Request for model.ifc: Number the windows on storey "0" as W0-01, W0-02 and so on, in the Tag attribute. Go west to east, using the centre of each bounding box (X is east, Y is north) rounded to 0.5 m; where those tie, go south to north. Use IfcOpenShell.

First a look at what the model holds.

```python
import ifcopenshell
import ifcopenshell.util.element
import ifcopenshell.util.placement

model = ifcopenshell.open("model.ifc")
print(model.schema)
storey = next(s for s in model.by_type("IfcBuildingStorey") if s.Name == "0")
windows = [e for e in ifcopenshell.util.element.get_decomposition(storey) if e.is_a("IfcWindow")]
for e in sorted(windows, key=lambda e: e.id()):
    origin = ifcopenshell.util.placement.get_local_placement(e.ObjectPlacement)[:3, 3]
    print(e.id(), e.Tag, e.Name, origin.round(2) + 0.0, sep=" | ")
```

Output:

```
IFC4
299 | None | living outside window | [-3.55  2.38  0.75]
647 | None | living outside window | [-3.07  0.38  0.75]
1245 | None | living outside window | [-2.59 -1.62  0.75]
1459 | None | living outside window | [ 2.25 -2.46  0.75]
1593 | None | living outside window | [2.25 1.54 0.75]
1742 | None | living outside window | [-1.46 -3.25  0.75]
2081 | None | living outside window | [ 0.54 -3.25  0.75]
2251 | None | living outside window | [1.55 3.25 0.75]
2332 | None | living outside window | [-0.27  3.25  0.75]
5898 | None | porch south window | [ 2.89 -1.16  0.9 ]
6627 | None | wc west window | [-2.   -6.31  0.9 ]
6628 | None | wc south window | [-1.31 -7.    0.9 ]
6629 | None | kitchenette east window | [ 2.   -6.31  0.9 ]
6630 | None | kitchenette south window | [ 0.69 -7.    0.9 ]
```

```python
import ifcopenshell
import ifcopenshell.geom
import ifcopenshell.util.element
import ifcopenshell.util.shape

model = ifcopenshell.open("model.ifc")
settings = ifcopenshell.geom.settings()
settings.set("use-world-coords", True)


def centre(element):
    shape = ifcopenshell.geom.create_shape(settings, element)
    return ifcopenshell.util.shape.get_bbox_centroid(shape.geometry)


storey = next(s for s in model.by_type("IfcBuildingStorey") if s.Name == "0")
windows = [e for e in ifcopenshell.util.element.get_decomposition(storey) if e.is_a("IfcWindow")]

# Insertion points can sit at a corner or the storey origin, so sort by the geometry (in metres).
centres = {e: centre(e) for e in windows}
windows.sort(key=lambda e: (round(centres[e][0] / 0.5), centres[e][1]))

for i, e in enumerate(windows, start=1):
    number = f"W0-{i:02d}"
    e.Tag = number
    print(e.id(), number)

model.write("model_v2.ifc")
```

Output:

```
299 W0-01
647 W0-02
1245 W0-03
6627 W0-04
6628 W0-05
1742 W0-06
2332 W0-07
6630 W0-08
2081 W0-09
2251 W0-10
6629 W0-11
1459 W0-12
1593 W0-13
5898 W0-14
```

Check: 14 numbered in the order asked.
